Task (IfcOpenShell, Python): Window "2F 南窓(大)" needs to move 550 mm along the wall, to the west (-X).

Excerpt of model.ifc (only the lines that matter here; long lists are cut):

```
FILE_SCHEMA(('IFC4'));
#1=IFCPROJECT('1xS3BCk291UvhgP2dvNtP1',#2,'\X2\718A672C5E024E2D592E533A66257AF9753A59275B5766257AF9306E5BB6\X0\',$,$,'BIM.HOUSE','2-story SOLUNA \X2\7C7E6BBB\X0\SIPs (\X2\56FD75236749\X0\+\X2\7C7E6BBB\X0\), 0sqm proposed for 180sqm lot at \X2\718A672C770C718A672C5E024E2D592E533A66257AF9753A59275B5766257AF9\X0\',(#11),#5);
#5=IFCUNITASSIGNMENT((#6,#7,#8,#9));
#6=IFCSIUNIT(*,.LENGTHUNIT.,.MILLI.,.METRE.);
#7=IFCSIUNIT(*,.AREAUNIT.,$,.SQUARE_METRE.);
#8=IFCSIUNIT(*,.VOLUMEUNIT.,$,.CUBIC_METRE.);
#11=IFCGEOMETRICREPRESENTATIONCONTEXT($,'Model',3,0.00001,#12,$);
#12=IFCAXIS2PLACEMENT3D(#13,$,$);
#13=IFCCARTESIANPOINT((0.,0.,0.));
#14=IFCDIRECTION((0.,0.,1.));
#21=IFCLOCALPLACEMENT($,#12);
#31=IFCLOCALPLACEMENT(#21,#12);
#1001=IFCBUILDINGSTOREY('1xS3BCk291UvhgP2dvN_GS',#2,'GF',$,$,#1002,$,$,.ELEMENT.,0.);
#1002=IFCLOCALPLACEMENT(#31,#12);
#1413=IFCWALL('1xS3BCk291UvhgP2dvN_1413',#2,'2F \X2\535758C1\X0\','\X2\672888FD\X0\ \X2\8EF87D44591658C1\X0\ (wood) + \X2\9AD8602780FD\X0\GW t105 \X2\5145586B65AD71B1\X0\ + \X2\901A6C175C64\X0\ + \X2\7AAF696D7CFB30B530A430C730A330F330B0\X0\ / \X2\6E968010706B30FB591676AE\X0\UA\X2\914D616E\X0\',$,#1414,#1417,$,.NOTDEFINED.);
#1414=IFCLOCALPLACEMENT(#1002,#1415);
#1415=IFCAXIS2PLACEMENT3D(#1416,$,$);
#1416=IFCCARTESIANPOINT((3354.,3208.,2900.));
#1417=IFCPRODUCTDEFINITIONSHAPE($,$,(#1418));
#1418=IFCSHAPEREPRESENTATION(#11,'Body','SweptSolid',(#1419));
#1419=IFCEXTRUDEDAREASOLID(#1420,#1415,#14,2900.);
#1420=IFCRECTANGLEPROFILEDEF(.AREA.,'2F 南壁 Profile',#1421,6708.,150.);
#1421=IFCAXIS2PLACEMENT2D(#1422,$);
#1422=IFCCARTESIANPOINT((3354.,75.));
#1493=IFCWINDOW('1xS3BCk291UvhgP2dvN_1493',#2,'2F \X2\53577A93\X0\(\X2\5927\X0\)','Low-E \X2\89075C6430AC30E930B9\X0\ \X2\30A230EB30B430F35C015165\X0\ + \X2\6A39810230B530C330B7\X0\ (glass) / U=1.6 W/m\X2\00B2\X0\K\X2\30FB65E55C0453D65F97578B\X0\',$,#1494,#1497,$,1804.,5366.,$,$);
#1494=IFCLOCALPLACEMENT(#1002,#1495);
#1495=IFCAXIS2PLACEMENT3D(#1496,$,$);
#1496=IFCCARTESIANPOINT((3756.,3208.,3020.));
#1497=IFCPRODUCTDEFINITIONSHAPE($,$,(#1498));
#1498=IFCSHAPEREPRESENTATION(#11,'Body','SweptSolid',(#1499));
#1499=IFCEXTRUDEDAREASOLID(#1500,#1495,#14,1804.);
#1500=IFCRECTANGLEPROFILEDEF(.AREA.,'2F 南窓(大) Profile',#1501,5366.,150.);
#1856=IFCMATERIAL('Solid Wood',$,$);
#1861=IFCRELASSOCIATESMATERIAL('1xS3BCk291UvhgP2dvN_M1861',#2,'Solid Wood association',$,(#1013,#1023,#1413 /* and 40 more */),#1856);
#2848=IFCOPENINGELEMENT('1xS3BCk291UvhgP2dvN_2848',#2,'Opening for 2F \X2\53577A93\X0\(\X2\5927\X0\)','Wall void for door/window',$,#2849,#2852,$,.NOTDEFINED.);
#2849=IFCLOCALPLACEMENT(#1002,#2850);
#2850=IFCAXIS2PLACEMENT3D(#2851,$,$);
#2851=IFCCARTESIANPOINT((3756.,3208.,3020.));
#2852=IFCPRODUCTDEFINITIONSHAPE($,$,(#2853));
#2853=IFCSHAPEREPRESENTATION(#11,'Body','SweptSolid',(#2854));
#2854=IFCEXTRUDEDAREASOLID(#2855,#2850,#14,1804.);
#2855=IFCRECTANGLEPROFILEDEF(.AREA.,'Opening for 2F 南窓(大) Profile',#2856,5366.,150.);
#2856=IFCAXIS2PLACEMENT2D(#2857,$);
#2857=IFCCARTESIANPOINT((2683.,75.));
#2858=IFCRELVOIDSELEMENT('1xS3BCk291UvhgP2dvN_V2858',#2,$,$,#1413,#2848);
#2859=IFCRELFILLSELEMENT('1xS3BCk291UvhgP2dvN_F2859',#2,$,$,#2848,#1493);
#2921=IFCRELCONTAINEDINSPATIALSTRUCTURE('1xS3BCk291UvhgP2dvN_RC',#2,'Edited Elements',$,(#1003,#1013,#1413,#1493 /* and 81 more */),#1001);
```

```python
import ifcopenshell
import ifcopenshell.api.geometry
import ifcopenshell.util.placement

model = ifcopenshell.open("model.ifc")

window = model.by_guid("1xS3BCk291UvhgP2dvN_1493")
opening = window.FillsVoids[0].RelatingOpeningElement
wall = opening.VoidsElements[0].RelatingBuildingElement

wall_matrix = ifcopenshell.util.placement.get_local_placement(wall.ObjectPlacement)
shift = wall_matrix[:3, 0] * -550.0
before = ifcopenshell.util.placement.get_local_placement(window.ObjectPlacement)[:3, 3].copy()

# The window is not placed relative to its opening, so move both.
for product in (opening, window):
    matrix = ifcopenshell.util.placement.get_local_placement(product.ObjectPlacement)
    matrix[:3, 3] += shift
    ifcopenshell.api.geometry.edit_object_placement(model, product=product, matrix=matrix, is_si=False)

after = ifcopenshell.util.placement.get_local_placement(window.ObjectPlacement)[:3, 3]
print("window moved by", (after - before).round(3) + 0.0)

model.write("model-out.ifc")
```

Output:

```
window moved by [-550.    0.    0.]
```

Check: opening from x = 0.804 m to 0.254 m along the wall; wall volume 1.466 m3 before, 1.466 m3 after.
